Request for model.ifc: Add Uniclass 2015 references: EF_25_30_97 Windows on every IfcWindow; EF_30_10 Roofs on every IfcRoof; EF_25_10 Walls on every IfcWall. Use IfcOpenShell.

First a look at what the model holds.

```python
import ifcopenshell

model = ifcopenshell.open("model.ifc")
print(model.schema)
print("classifications:", [c.Name for c in model.by_type("IfcClassification")])
for ifc_class in ("IfcDoor", "IfcRoof", "IfcStair", "IfcWall", "IfcWindow"):
    print(ifc_class, len(model.by_type(ifc_class)))
```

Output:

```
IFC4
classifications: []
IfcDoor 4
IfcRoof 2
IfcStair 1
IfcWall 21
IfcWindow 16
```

```python
import ifcopenshell
import ifcopenshell.api.classification

model = ifcopenshell.open("model.ifc")

system = ifcopenshell.api.classification.add_classification(model, classification="Uniclass 2015")

codes = {
    "IfcWindow": ("EF_25_30_97", "Windows"),
    "IfcRoof": ("EF_30_10", "Roofs"),
    "IfcWall": ("EF_25_10", "Walls"),
}
for ifc_class, (code, name) in codes.items():
    products = model.by_type(ifc_class)
    ifcopenshell.api.classification.add_reference(
        model, products=products, classification=system, identification=code, name=name
    )
    print(code, len(products))

model.write("model_rev.ifc")
```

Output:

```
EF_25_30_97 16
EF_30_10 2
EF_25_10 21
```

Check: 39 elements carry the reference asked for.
